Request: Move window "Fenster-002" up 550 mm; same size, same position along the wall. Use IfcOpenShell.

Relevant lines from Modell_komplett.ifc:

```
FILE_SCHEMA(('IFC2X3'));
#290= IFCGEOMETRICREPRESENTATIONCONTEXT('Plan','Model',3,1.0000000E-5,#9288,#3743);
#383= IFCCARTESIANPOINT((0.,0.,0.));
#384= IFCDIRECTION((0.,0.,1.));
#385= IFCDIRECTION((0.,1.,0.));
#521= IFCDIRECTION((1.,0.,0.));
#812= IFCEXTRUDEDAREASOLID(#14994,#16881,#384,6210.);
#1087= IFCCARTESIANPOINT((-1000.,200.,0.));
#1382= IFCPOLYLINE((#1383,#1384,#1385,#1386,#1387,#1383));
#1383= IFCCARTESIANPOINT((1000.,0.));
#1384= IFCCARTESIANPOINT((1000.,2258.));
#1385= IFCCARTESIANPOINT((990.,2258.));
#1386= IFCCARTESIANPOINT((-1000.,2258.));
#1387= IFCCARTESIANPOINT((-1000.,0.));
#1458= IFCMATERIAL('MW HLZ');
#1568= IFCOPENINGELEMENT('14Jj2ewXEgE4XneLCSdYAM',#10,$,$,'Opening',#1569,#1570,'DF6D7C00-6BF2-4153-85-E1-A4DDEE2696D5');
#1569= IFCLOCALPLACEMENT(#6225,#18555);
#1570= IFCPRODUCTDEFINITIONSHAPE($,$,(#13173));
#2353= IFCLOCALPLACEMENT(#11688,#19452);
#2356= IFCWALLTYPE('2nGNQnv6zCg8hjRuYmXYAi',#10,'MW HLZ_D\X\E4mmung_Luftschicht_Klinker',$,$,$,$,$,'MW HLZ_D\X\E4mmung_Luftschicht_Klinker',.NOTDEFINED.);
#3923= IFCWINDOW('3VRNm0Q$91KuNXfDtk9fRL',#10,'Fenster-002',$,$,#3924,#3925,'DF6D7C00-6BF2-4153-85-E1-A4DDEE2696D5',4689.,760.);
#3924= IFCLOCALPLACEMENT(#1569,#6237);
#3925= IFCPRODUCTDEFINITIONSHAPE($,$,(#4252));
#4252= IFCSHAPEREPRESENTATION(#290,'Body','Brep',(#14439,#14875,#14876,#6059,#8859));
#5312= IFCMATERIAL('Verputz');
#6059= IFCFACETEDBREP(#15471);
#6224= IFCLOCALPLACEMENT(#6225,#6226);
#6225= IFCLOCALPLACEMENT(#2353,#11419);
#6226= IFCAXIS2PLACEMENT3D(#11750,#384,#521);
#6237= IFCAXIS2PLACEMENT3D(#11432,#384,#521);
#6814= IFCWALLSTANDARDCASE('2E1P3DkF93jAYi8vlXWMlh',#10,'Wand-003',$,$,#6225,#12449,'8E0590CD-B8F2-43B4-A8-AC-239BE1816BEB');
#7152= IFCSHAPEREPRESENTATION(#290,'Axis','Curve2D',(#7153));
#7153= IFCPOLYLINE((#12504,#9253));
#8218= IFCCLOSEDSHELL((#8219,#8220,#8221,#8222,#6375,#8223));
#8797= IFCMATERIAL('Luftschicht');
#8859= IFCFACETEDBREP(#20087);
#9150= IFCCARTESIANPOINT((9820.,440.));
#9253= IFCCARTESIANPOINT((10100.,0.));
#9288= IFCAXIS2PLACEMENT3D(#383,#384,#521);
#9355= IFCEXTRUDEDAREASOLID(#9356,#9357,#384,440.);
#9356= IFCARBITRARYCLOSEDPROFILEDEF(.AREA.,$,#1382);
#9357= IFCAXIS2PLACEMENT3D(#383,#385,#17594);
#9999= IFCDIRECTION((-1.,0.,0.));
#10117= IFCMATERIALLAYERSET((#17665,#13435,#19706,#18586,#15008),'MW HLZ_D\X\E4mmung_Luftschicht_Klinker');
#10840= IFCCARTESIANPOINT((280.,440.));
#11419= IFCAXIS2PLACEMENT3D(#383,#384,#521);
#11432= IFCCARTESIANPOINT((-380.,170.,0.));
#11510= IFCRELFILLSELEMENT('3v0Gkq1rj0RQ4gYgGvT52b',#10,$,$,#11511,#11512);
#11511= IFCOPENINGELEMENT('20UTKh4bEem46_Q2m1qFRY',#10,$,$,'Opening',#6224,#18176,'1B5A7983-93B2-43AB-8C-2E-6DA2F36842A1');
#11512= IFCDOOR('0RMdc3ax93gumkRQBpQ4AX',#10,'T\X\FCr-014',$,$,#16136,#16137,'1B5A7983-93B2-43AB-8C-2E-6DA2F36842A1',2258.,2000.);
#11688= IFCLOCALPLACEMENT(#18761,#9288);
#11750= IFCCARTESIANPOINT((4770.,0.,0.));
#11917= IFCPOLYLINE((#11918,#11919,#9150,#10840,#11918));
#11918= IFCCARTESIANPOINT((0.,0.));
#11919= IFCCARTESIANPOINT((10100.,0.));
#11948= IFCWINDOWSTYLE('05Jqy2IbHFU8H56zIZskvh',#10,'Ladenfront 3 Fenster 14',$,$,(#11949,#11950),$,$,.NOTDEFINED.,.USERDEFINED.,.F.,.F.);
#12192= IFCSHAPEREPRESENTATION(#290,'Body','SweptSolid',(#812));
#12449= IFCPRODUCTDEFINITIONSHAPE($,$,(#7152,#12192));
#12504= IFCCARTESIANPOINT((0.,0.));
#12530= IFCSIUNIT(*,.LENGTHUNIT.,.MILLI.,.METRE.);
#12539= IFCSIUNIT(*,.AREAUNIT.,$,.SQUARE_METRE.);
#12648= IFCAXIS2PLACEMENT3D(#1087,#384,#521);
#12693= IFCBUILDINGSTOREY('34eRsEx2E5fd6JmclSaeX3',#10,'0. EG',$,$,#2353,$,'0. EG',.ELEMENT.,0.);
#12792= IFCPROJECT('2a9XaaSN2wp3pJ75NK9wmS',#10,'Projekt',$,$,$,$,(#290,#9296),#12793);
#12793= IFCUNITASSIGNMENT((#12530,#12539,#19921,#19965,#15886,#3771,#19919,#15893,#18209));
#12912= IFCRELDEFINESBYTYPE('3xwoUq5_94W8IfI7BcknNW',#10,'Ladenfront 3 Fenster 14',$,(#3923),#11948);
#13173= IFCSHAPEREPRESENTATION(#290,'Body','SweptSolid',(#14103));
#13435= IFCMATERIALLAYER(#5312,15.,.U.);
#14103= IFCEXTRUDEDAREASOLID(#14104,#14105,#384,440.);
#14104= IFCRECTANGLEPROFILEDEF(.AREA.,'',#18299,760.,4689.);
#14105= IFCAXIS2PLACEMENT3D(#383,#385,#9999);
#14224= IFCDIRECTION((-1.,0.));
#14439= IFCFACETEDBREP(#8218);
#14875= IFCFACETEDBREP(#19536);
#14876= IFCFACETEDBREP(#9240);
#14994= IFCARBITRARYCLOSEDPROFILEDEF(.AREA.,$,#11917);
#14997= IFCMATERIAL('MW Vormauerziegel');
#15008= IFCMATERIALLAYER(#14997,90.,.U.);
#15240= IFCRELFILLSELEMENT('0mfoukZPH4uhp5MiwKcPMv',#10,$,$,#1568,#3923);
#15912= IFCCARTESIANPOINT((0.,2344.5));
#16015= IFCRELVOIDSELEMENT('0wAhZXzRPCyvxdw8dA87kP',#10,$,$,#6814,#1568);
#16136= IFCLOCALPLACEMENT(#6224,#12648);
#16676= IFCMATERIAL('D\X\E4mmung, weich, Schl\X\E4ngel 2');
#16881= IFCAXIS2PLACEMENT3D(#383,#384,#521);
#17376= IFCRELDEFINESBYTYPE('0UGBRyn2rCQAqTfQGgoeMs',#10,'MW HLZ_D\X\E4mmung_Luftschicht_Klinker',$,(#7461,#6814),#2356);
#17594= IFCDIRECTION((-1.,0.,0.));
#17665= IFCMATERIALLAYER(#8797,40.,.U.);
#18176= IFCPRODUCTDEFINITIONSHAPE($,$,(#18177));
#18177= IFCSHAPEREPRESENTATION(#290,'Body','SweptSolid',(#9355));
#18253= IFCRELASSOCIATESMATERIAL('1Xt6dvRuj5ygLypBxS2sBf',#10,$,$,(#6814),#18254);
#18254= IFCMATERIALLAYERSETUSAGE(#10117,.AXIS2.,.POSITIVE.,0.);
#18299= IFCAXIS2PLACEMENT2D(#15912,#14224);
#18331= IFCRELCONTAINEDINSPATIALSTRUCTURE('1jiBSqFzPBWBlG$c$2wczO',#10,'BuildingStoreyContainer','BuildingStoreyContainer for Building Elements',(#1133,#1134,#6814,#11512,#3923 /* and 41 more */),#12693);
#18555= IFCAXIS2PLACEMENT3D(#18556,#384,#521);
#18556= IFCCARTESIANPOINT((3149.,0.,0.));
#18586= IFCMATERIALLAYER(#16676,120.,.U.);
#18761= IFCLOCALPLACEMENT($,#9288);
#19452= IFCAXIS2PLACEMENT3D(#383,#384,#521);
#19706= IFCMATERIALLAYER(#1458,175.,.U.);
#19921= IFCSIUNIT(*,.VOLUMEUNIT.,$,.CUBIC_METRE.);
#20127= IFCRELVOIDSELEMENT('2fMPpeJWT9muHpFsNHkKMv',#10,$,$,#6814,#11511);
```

```python
import numpy as np
import ifcopenshell
import ifcopenshell.api.geometry
import ifcopenshell.util.placement
import ifcopenshell.util.unit

model = ifcopenshell.open("Modell_komplett.ifc")
unit_scale = ifcopenshell.util.unit.calculate_unit_scale(model)

window = model.by_guid("3VRNm0Q$91KuNXfDtk9fRL")
opening = window.FillsVoids[0].RelatingOpeningElement
dz = 0.55 / unit_scale

shift = np.array([0.0, 0.0, dz])
# The window is placed relative to its opening, so it follows when the opening moves.
matrix = ifcopenshell.util.placement.get_local_placement(opening.ObjectPlacement)
matrix[:3, 3] += shift
ifcopenshell.api.geometry.edit_object_placement(
    model, product=opening, matrix=matrix, is_si=False, should_transform_children=True
)

print(f"moved by {dz * unit_scale:+.3f} m")

model.write("Modell_komplett_v2.ifc")
```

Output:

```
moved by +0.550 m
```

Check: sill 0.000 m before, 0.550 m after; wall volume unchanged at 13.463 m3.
